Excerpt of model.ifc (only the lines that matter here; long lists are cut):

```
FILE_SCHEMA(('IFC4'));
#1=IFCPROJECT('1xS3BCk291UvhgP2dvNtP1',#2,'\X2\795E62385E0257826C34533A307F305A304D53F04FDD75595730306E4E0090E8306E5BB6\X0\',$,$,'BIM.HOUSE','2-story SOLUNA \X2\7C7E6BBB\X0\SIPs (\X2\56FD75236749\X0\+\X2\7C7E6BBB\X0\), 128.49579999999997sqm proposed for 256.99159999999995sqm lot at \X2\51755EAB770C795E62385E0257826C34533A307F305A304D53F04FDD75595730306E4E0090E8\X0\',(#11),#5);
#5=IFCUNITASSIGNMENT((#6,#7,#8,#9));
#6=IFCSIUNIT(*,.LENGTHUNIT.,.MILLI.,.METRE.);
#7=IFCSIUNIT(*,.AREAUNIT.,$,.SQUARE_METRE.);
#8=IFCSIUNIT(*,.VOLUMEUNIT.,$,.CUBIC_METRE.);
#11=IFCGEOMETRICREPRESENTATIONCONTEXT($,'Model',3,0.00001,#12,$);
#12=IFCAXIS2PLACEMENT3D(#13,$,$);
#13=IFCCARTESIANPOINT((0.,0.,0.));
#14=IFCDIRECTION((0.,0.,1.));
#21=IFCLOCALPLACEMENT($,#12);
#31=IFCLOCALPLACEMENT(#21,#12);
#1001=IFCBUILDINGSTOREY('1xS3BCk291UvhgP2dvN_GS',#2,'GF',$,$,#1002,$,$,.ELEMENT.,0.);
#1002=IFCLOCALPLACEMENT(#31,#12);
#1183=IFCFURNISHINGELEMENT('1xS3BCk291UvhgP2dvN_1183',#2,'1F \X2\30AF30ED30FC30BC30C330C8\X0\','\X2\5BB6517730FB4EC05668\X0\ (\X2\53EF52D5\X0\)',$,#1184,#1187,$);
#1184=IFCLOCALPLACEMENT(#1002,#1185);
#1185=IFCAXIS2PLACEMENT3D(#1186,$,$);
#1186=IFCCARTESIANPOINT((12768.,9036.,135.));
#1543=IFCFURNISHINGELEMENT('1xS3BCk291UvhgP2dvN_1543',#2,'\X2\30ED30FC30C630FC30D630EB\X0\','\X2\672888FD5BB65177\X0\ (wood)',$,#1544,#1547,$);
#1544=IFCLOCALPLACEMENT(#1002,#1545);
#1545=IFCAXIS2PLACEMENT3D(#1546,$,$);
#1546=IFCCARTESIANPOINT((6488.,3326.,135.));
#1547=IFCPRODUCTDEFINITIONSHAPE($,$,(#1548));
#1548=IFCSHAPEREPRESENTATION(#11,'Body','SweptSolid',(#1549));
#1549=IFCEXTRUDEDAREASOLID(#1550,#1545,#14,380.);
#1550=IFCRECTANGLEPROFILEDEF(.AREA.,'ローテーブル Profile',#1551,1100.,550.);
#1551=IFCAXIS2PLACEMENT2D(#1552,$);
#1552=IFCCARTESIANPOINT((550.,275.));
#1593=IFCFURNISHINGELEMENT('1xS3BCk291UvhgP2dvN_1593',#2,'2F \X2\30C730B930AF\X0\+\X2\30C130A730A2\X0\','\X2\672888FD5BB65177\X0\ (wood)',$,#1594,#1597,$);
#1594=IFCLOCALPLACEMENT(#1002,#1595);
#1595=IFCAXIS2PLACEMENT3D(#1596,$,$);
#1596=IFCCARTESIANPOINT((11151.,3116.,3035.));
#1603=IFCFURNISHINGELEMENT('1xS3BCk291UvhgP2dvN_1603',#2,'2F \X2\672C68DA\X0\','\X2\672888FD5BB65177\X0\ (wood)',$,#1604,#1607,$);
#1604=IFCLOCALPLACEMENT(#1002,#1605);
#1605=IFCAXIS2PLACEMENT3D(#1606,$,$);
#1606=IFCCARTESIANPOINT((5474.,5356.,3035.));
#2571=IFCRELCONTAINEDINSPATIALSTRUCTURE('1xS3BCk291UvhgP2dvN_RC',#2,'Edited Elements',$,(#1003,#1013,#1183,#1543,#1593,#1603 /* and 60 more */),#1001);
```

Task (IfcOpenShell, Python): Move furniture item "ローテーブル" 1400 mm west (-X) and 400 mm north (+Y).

```python
import ifcopenshell
import ifcopenshell.api.geometry
import ifcopenshell.util.placement
import ifcopenshell.util.unit

model = ifcopenshell.open("model.ifc")
unit_scale = ifcopenshell.util.unit.calculate_unit_scale(model)

item = model.by_id(1543)
matrix = ifcopenshell.util.placement.get_local_placement(item.ObjectPlacement)
matrix[0, 3] -= 1.4 / unit_scale
matrix[1, 3] += 0.4 / unit_scale
ifcopenshell.api.geometry.edit_object_placement(model, product=item, matrix=matrix, is_si=False)

print(ifcopenshell.util.placement.get_local_placement(item.ObjectPlacement).round(3) + 0.0)

model.write("model_updated.ifc")
```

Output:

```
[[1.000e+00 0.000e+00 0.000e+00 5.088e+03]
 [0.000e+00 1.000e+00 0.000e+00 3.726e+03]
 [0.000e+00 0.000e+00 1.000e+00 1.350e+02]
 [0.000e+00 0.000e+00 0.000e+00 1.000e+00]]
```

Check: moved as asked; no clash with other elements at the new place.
